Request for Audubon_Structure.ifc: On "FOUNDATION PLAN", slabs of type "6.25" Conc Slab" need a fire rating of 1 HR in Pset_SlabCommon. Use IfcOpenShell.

First a look at what the model holds.

```python
import ifcopenshell
import ifcopenshell.util.element

model = ifcopenshell.open("Audubon_Structure.ifc")
print(model.schema)
storey = next(s for s in model.by_type("IfcBuildingStorey") if s.Name == "FOUNDATION PLAN")
slabs = [e for e in ifcopenshell.util.element.get_decomposition(storey) if e.is_a("IfcSlab")]
seen = {}
for e in slabs:
    element_type = ifcopenshell.util.element.get_type(e)
    key = (element_type.Name if element_type != e and element_type else None, ifcopenshell.util.element.get_pset(e, "Pset_SlabCommon", "FireRating"))
    seen[key] = seen.get(key, 0) + 1
for (name, value), count in sorted(seen.items(), key=str):
    print(count, "x", name, "|", value)
```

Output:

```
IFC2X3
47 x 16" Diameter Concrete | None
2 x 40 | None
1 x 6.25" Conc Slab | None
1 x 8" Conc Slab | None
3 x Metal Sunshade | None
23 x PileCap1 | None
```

```python
import ifcopenshell
import ifcopenshell.api.pset
import ifcopenshell.util.element

model = ifcopenshell.open("Audubon_Structure.ifc")

storey = next(s for s in model.by_type("IfcBuildingStorey") if s.Name == "FOUNDATION PLAN")
slabs = [e for e in ifcopenshell.util.element.get_decomposition(storey) if e.is_a("IfcSlab")]

count = 0
for e in slabs:
    element_type = ifcopenshell.util.element.get_type(e)
    if element_type in (None, e) or element_type.Name != '6.25" Conc Slab':
        continue
    # add_pset returns the element's existing set when there is one.
    pset = ifcopenshell.api.pset.add_pset(model, product=e, name="Pset_SlabCommon")
    ifcopenshell.api.pset.edit_pset(model, pset=pset, properties={"FireRating": "1 HR"})
    count += 1

print(count, "slabs updated")

model.write("Audubon_Structure-out.ifc")
```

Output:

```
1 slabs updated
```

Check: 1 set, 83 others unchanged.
